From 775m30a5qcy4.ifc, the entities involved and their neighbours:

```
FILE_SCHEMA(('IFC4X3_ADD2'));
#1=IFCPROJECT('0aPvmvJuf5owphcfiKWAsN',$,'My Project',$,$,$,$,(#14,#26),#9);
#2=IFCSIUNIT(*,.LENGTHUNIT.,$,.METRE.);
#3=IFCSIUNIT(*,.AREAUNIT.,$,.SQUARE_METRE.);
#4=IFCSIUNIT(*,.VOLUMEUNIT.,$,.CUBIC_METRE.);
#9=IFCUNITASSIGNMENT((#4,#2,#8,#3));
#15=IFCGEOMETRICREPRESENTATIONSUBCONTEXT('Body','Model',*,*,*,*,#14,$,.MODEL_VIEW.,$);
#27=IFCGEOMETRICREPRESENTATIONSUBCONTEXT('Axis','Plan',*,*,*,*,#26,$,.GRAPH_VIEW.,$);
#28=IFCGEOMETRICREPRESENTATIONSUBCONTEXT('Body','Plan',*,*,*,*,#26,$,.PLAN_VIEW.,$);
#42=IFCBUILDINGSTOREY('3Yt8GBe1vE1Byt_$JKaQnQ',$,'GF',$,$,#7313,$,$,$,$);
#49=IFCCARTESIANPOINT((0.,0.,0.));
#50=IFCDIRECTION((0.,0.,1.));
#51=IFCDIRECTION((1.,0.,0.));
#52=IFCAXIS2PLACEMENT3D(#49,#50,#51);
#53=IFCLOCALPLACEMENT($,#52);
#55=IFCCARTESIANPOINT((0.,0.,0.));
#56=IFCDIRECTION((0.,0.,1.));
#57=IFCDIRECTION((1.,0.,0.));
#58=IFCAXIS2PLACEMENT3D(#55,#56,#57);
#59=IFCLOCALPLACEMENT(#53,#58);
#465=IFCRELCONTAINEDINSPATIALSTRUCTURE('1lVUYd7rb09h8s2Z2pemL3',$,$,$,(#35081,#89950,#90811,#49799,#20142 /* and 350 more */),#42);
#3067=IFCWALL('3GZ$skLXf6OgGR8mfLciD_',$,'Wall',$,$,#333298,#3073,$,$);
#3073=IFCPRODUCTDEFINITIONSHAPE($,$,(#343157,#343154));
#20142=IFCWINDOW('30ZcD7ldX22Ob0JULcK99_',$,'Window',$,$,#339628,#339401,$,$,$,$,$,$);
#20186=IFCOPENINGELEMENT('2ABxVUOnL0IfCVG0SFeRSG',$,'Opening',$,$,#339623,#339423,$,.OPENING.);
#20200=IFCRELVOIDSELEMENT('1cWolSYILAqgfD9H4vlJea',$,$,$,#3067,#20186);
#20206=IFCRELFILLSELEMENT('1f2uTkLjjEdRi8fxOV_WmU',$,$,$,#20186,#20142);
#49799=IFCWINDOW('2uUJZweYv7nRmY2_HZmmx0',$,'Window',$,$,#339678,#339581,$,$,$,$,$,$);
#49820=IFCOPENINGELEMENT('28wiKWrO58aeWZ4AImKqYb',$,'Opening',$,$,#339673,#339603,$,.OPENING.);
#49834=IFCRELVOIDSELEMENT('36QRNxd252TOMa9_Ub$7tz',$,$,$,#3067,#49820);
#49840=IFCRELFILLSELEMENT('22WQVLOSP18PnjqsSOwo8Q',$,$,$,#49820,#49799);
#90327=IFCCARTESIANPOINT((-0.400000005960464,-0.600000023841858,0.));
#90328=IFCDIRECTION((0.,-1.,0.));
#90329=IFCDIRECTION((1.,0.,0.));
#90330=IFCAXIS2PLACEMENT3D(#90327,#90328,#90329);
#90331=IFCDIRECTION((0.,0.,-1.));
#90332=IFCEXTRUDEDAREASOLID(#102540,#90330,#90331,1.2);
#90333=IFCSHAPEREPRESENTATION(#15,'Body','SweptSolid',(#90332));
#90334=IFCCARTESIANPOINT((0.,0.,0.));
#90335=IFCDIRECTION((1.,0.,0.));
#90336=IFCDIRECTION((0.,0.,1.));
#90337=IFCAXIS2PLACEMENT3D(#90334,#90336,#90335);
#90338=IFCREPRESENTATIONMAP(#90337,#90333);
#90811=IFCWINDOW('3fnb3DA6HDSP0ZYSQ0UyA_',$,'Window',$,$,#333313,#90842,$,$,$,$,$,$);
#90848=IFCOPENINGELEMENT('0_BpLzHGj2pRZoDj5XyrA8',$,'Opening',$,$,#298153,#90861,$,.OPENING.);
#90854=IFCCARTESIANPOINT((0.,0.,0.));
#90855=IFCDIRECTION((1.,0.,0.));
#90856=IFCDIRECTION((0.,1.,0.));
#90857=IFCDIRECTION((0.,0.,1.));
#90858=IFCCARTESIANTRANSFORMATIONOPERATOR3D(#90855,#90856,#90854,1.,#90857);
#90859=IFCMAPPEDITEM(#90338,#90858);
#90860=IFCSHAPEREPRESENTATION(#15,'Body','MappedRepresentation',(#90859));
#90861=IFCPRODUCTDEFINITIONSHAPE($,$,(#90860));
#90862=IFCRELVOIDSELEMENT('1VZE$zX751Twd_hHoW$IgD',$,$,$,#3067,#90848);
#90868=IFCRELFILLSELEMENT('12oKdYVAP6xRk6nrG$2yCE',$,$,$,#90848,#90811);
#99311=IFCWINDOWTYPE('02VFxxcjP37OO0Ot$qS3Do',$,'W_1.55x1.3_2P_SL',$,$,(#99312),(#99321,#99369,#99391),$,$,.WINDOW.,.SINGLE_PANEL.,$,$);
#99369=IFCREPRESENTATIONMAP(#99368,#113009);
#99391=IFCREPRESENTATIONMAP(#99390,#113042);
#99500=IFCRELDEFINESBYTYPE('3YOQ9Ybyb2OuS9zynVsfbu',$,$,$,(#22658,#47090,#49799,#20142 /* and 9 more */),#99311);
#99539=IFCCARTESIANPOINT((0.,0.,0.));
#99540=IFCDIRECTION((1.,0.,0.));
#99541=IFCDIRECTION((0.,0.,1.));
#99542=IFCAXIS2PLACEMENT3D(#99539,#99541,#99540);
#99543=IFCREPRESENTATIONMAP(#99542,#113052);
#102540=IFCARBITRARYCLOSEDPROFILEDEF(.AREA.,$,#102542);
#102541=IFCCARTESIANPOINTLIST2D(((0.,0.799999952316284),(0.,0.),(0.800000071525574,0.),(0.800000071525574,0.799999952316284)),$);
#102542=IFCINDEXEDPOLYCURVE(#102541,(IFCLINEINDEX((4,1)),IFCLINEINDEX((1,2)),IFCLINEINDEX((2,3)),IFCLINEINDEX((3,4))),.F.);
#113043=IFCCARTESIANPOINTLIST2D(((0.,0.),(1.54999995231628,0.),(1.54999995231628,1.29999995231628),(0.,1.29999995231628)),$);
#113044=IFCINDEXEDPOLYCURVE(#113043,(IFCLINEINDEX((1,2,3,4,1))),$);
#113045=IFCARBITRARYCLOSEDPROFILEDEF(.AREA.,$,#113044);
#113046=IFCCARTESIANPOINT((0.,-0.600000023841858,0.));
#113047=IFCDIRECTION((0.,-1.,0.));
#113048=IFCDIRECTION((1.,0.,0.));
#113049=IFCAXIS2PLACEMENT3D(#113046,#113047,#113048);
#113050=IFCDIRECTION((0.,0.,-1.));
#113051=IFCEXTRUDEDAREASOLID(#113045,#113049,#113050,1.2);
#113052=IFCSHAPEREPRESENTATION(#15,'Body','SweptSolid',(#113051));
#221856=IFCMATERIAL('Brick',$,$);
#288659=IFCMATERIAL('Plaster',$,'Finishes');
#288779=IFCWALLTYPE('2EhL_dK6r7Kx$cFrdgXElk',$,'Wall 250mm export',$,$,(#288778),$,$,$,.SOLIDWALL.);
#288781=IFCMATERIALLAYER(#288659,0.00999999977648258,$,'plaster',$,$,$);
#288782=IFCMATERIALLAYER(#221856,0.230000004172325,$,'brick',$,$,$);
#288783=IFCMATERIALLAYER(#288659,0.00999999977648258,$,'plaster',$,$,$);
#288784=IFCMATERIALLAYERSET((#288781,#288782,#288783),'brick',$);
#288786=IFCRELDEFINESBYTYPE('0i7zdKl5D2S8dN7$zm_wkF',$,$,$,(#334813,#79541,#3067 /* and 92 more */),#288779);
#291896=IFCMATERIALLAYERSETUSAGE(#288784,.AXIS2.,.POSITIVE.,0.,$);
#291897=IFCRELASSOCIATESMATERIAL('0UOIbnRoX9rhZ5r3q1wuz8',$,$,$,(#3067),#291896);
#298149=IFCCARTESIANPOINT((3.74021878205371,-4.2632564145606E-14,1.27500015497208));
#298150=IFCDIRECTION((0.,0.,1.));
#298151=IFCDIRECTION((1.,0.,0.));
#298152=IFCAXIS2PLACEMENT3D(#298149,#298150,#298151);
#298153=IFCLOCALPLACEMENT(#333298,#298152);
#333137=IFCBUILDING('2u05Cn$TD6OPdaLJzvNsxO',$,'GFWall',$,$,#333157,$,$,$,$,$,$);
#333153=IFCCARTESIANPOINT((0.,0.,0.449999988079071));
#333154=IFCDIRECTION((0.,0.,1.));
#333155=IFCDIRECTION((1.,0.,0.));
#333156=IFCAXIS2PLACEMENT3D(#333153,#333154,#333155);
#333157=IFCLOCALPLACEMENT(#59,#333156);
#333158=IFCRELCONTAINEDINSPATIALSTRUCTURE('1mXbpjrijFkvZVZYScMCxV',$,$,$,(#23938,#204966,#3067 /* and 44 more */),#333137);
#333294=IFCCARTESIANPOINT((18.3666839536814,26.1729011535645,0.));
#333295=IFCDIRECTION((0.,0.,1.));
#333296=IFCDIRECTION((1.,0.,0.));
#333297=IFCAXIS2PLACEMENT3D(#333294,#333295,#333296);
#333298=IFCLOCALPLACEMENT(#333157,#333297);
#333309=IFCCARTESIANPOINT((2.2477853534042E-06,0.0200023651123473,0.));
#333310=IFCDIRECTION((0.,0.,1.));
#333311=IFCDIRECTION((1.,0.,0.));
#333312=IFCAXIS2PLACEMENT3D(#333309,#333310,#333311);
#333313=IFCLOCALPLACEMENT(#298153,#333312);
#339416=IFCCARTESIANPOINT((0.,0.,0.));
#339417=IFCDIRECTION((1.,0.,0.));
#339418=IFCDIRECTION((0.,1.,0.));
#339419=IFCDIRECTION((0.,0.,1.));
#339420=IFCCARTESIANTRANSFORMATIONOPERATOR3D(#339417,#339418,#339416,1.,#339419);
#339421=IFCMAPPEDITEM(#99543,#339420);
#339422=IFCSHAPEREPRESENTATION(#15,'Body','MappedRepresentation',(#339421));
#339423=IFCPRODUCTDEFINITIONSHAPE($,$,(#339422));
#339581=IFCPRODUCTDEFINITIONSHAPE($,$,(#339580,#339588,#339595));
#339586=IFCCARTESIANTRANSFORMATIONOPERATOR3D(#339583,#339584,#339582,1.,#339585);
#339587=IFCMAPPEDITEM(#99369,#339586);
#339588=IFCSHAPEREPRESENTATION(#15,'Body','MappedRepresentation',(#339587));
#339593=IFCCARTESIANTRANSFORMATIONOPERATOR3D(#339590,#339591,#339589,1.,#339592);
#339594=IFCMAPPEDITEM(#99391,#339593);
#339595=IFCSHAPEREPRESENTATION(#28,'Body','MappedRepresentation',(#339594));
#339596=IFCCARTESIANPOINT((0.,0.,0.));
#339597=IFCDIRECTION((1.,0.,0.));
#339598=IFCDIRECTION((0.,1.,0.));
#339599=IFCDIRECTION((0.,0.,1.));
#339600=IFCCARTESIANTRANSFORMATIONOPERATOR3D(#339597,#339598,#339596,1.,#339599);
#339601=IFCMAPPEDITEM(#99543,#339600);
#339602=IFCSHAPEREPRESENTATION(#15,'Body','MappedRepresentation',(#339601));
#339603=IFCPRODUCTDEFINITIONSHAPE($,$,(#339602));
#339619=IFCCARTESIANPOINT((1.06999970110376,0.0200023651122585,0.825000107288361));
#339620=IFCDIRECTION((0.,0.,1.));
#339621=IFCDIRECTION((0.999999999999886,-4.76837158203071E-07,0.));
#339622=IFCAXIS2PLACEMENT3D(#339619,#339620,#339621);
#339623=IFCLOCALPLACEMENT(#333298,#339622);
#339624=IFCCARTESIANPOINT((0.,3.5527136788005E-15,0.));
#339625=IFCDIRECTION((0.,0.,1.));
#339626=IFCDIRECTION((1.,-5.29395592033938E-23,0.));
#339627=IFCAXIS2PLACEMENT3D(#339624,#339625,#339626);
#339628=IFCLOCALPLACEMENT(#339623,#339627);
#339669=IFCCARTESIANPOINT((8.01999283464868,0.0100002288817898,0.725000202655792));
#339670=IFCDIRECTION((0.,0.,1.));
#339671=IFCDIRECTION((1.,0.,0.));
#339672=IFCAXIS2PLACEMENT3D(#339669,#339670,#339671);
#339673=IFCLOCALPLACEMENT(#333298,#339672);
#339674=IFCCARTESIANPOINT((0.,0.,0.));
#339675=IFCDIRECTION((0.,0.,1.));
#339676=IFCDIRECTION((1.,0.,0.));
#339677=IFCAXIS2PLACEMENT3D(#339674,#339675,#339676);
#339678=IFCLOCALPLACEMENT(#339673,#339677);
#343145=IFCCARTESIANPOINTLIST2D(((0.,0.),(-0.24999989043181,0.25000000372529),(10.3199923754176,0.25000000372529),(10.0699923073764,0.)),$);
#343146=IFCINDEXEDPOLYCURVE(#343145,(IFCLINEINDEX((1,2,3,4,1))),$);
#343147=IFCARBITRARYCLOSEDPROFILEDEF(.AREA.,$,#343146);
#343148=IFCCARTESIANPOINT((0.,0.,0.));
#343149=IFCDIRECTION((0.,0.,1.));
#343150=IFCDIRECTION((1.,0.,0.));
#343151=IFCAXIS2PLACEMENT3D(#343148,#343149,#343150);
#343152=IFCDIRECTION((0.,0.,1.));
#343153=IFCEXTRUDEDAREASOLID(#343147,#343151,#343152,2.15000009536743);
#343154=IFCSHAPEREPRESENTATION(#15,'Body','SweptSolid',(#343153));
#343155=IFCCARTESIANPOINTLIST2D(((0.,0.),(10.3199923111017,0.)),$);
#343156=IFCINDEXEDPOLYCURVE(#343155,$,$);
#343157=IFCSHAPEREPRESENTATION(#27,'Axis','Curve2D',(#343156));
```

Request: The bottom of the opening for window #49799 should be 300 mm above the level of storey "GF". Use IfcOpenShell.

```python
import numpy as np
import ifcopenshell
import ifcopenshell.api.geometry
import ifcopenshell.geom
import ifcopenshell.util.element
import ifcopenshell.util.placement
import ifcopenshell.util.shape
import ifcopenshell.util.unit

model = ifcopenshell.open("775m30a5qcy4.ifc")
unit_scale = ifcopenshell.util.unit.calculate_unit_scale(model)

window = model.by_guid("2uUJZweYv7nRmY2_HZmmx0")
opening = window.FillsVoids[0].RelatingOpeningElement
storey = ifcopenshell.util.element.get_container(window, ifc_class="IfcBuildingStorey")
level = ifcopenshell.util.placement.get_local_placement(storey.ObjectPlacement)[2, 3]

# The opening's origin need not be at the sill, so measure its lowest point.
shape = ifcopenshell.geom.create_shape(ifcopenshell.geom.settings(), opening)
bottom = ifcopenshell.util.shape.get_shape_bottom_elevation(shape, shape.geometry) / unit_scale
dz = level + 0.3 - bottom

shift = np.array([0.0, 0.0, dz])
# The window is placed relative to its opening, so it follows when the opening moves.
matrix = ifcopenshell.util.placement.get_local_placement(opening.ObjectPlacement)
matrix[:3, 3] += shift
ifcopenshell.api.geometry.edit_object_placement(
    model, product=opening, matrix=matrix, is_si=False, should_transform_children=True
)

print(f"moved by {dz * unit_scale:+.3f} m")

model.write("775m30a5qcy4-out.ifc")
```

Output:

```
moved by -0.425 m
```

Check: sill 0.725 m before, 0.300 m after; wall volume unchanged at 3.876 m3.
